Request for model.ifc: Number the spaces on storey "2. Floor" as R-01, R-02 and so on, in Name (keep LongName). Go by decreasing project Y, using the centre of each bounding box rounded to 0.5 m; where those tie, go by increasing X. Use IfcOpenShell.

First a look at what the model holds.

```python
import ifcopenshell
import ifcopenshell.util.element
import ifcopenshell.util.placement

model = ifcopenshell.open("model.ifc")
print(model.schema)
storey = next(s for s in model.by_type("IfcBuildingStorey") if s.Name == "2. Floor")
spaces = [e for e in ifcopenshell.util.element.get_decomposition(storey) if e.is_a("IfcSpace")]
for e in sorted(spaces, key=lambda e: e.id()):
    origin = ifcopenshell.util.placement.get_local_placement(e.ObjectPlacement)[:3, 3]
    print(e.id(), e.Name, e.LongName, origin.round(2) + 0.0, sep=" | ")
```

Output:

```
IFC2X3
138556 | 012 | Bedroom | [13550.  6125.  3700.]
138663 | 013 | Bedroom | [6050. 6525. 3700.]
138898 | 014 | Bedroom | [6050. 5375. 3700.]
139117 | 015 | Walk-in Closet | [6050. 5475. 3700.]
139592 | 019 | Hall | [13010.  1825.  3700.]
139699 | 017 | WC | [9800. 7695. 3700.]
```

```python
import ifcopenshell
import ifcopenshell.geom
import ifcopenshell.util.element
import ifcopenshell.util.shape

model = ifcopenshell.open("model.ifc")
settings = ifcopenshell.geom.settings()
settings.set("use-world-coords", True)


def centre(element):
    shape = ifcopenshell.geom.create_shape(settings, element)
    return ifcopenshell.util.shape.get_bbox_centroid(shape.geometry)


storey = next(s for s in model.by_type("IfcBuildingStorey") if s.Name == "2. Floor")
spaces = [e for e in ifcopenshell.util.element.get_decomposition(storey) if e.is_a("IfcSpace")]

# Insertion points can sit at a corner or the storey origin, so sort by the geometry (in metres).
centres = {e: centre(e) for e in spaces}
spaces.sort(key=lambda e: (-round(centres[e][1] / 0.5), centres[e][0]))

for i, e in enumerate(spaces, start=1):
    number = f"R-{i:02d}"
    e.Name = number
    print(e.id(), number)

model.write("model_edited.ifc")
```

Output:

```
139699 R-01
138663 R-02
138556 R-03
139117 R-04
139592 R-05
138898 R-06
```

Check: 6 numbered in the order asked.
